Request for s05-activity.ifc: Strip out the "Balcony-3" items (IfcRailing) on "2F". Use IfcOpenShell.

First a look at what the model holds.

```python
import ifcopenshell
import ifcopenshell.util.element

model = ifcopenshell.open("s05-activity.ifc")
print(model.schema)
storey = next(s for s in model.by_type("IfcBuildingStorey") if s.Name == "2F")
railings = [e for e in ifcopenshell.util.element.get_decomposition(storey) if e.is_a("IfcRailing")]
seen = {}
for e in railings:
    element_type = ifcopenshell.util.element.get_type(e)
    name = element_type.Name if element_type not in (None, e) else None
    seen[name] = seen.get(name, 0) + 1
for name, count in sorted(seen.items(), key=str):
    print(count, "x", name)
```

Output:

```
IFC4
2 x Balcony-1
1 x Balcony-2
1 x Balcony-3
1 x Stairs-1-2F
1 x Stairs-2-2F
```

```python
import ifcopenshell
import ifcopenshell.api.root
import ifcopenshell.util.element

model = ifcopenshell.open("s05-activity.ifc")

storey = next(s for s in model.by_type("IfcBuildingStorey") if s.Name == "2F")
railings = [e for e in ifcopenshell.util.element.get_decomposition(storey) if e.is_a("IfcRailing")]
targets = [e for e in railings if (t := ifcopenshell.util.element.get_type(e)) not in (None, e) and t.Name == "Balcony-3"]

for e in targets:
    ifcopenshell.api.root.remove_product(model, product=e)
print(len(targets), "removed")

model.write("s05-activity_updated.ifc")
```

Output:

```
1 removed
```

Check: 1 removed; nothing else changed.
